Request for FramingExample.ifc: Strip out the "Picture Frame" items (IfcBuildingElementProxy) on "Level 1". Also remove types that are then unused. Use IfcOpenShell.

First a look at what the model holds.

```python
import ifcopenshell
import ifcopenshell.util.element

model = ifcopenshell.open("FramingExample.ifc")
print(model.schema)
storey = next(s for s in model.by_type("IfcBuildingStorey") if s.Name == "Level 1")
proxies = [e for e in ifcopenshell.util.element.get_decomposition(storey) if e.is_a("IfcBuildingElementProxy")]
seen = {}
for e in proxies:
    element_type = ifcopenshell.util.element.get_type(e)
    name = element_type.Name if element_type not in (None, e) else None
    seen[name] = seen.get(name, 0) + 1
for name, count in sorted(seen.items(), key=str):
    print(count, "x", name)
```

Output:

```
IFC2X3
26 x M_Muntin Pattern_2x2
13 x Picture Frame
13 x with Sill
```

```python
import ifcopenshell
import ifcopenshell.api.root
import ifcopenshell.util.element

model = ifcopenshell.open("FramingExample.ifc")

storey = next(s for s in model.by_type("IfcBuildingStorey") if s.Name == "Level 1")
proxies = [e for e in ifcopenshell.util.element.get_decomposition(storey) if e.is_a("IfcBuildingElementProxy")]
targets = [e for e in proxies if (t := ifcopenshell.util.element.get_type(e)) not in (None, e) and t.Name == "Picture Frame"]
types = {ifcopenshell.util.element.get_type(e) for e in targets} - {None, *targets}

for e in targets:
    ifcopenshell.api.root.remove_product(model, product=e)
print(len(targets), "removed")

unused = [t for t in types if not ifcopenshell.util.element.get_types(t)]
for t in unused:
    ifcopenshell.api.root.remove_product(model, product=t)
print(len(unused), "unused types removed")

model.write("FramingExample-out.ifc")
```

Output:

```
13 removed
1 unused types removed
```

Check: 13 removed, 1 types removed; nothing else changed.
